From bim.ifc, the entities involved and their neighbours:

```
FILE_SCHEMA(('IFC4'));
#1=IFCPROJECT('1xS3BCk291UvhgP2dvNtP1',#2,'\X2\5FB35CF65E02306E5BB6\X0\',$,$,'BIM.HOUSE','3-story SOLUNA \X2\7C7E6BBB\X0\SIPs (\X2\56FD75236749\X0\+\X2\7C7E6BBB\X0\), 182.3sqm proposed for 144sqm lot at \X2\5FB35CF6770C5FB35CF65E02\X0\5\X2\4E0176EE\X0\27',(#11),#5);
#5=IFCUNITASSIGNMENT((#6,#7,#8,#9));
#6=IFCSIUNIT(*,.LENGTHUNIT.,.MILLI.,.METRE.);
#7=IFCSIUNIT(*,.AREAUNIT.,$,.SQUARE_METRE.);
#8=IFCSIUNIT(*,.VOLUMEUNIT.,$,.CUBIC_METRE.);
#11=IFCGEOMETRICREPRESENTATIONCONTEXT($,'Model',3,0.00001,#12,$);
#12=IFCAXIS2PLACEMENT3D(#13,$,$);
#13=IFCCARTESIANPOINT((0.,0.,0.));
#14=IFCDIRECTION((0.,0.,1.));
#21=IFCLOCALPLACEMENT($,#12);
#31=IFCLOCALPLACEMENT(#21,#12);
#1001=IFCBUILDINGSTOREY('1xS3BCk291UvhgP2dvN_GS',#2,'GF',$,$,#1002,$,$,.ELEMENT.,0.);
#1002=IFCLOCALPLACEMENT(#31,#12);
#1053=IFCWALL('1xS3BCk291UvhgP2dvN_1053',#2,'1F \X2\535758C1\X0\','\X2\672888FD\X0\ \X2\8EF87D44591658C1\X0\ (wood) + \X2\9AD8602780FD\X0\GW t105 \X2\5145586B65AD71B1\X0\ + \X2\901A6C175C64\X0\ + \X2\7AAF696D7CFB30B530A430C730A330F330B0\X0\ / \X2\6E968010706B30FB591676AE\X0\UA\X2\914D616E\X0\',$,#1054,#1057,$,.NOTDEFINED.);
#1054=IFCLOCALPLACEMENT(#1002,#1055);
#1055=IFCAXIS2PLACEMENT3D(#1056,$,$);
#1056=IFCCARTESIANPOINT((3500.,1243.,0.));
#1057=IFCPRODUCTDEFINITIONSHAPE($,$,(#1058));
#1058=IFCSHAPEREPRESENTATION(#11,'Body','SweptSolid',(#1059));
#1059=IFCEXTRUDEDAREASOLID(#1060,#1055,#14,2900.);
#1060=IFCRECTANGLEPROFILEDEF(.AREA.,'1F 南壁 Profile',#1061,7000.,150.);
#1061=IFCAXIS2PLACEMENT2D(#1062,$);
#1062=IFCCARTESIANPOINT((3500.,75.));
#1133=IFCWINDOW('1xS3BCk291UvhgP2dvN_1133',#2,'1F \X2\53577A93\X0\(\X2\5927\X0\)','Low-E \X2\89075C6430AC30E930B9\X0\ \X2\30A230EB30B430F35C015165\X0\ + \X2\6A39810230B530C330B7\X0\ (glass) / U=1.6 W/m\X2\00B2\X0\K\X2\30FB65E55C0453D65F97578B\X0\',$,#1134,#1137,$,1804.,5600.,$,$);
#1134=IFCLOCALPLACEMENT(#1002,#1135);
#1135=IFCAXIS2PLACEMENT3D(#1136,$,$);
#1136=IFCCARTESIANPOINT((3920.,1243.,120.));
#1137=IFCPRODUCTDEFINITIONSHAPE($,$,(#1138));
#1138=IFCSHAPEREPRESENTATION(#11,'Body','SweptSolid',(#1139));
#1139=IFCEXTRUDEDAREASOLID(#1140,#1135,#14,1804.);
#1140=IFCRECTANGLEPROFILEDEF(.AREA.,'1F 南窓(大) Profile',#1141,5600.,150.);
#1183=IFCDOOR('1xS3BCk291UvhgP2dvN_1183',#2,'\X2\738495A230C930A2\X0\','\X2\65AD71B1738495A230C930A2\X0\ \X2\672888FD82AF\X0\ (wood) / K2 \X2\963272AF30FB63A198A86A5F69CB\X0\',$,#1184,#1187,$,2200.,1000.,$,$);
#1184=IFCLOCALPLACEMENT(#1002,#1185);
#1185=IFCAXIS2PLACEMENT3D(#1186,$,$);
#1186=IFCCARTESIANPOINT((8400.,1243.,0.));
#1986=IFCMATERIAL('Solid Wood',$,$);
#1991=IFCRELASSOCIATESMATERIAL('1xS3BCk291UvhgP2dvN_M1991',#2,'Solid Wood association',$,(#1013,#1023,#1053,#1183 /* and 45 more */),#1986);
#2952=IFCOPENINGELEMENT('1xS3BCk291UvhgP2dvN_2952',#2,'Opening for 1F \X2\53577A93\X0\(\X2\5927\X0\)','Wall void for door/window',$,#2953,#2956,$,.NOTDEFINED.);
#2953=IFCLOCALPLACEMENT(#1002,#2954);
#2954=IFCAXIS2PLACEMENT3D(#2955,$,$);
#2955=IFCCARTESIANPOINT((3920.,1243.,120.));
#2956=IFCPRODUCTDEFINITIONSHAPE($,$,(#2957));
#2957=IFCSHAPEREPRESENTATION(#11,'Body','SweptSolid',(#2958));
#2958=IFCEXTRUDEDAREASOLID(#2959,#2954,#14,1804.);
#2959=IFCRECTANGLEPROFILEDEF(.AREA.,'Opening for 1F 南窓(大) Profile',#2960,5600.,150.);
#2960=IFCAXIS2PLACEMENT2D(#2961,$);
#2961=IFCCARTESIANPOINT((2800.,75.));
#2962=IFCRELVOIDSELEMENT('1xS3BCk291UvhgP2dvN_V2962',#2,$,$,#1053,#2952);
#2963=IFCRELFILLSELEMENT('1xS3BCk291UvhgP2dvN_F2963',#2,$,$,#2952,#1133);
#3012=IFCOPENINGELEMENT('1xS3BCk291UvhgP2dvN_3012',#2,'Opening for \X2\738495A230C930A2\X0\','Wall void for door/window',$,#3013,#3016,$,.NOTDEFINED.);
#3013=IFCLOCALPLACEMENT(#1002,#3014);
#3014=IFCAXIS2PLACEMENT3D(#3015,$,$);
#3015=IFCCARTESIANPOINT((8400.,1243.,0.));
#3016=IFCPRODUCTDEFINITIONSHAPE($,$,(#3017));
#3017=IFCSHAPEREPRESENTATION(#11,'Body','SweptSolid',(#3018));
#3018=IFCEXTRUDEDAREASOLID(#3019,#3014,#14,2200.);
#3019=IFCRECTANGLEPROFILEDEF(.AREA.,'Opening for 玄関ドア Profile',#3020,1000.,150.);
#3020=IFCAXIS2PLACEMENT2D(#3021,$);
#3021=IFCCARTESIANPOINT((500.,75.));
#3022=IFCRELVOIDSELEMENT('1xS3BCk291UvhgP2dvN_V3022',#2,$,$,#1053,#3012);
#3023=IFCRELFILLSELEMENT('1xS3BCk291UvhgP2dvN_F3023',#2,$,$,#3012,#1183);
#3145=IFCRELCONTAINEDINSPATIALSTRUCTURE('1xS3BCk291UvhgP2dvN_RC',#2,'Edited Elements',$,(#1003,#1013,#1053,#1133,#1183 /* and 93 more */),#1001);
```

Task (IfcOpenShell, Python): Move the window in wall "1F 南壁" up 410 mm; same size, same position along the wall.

```python
import numpy as np
import ifcopenshell
import ifcopenshell.api.geometry
import ifcopenshell.util.placement
import ifcopenshell.util.unit

model = ifcopenshell.open("bim.ifc")
unit_scale = ifcopenshell.util.unit.calculate_unit_scale(model)

window = model.by_id(1133)
opening = window.FillsVoids[0].RelatingOpeningElement
dz = 410.0

shift = np.array([0.0, 0.0, dz])
# The window is not placed relative to its opening, so move both.
for product in (opening, window):
    matrix = ifcopenshell.util.placement.get_local_placement(product.ObjectPlacement)
    matrix[:3, 3] += shift
    ifcopenshell.api.geometry.edit_object_placement(model, product=product, matrix=matrix, is_si=False)

print(f"moved by {dz * unit_scale:+.3f} m")

model.write("bim-out.ifc")
```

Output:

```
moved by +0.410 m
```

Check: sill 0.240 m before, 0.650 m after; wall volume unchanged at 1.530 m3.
